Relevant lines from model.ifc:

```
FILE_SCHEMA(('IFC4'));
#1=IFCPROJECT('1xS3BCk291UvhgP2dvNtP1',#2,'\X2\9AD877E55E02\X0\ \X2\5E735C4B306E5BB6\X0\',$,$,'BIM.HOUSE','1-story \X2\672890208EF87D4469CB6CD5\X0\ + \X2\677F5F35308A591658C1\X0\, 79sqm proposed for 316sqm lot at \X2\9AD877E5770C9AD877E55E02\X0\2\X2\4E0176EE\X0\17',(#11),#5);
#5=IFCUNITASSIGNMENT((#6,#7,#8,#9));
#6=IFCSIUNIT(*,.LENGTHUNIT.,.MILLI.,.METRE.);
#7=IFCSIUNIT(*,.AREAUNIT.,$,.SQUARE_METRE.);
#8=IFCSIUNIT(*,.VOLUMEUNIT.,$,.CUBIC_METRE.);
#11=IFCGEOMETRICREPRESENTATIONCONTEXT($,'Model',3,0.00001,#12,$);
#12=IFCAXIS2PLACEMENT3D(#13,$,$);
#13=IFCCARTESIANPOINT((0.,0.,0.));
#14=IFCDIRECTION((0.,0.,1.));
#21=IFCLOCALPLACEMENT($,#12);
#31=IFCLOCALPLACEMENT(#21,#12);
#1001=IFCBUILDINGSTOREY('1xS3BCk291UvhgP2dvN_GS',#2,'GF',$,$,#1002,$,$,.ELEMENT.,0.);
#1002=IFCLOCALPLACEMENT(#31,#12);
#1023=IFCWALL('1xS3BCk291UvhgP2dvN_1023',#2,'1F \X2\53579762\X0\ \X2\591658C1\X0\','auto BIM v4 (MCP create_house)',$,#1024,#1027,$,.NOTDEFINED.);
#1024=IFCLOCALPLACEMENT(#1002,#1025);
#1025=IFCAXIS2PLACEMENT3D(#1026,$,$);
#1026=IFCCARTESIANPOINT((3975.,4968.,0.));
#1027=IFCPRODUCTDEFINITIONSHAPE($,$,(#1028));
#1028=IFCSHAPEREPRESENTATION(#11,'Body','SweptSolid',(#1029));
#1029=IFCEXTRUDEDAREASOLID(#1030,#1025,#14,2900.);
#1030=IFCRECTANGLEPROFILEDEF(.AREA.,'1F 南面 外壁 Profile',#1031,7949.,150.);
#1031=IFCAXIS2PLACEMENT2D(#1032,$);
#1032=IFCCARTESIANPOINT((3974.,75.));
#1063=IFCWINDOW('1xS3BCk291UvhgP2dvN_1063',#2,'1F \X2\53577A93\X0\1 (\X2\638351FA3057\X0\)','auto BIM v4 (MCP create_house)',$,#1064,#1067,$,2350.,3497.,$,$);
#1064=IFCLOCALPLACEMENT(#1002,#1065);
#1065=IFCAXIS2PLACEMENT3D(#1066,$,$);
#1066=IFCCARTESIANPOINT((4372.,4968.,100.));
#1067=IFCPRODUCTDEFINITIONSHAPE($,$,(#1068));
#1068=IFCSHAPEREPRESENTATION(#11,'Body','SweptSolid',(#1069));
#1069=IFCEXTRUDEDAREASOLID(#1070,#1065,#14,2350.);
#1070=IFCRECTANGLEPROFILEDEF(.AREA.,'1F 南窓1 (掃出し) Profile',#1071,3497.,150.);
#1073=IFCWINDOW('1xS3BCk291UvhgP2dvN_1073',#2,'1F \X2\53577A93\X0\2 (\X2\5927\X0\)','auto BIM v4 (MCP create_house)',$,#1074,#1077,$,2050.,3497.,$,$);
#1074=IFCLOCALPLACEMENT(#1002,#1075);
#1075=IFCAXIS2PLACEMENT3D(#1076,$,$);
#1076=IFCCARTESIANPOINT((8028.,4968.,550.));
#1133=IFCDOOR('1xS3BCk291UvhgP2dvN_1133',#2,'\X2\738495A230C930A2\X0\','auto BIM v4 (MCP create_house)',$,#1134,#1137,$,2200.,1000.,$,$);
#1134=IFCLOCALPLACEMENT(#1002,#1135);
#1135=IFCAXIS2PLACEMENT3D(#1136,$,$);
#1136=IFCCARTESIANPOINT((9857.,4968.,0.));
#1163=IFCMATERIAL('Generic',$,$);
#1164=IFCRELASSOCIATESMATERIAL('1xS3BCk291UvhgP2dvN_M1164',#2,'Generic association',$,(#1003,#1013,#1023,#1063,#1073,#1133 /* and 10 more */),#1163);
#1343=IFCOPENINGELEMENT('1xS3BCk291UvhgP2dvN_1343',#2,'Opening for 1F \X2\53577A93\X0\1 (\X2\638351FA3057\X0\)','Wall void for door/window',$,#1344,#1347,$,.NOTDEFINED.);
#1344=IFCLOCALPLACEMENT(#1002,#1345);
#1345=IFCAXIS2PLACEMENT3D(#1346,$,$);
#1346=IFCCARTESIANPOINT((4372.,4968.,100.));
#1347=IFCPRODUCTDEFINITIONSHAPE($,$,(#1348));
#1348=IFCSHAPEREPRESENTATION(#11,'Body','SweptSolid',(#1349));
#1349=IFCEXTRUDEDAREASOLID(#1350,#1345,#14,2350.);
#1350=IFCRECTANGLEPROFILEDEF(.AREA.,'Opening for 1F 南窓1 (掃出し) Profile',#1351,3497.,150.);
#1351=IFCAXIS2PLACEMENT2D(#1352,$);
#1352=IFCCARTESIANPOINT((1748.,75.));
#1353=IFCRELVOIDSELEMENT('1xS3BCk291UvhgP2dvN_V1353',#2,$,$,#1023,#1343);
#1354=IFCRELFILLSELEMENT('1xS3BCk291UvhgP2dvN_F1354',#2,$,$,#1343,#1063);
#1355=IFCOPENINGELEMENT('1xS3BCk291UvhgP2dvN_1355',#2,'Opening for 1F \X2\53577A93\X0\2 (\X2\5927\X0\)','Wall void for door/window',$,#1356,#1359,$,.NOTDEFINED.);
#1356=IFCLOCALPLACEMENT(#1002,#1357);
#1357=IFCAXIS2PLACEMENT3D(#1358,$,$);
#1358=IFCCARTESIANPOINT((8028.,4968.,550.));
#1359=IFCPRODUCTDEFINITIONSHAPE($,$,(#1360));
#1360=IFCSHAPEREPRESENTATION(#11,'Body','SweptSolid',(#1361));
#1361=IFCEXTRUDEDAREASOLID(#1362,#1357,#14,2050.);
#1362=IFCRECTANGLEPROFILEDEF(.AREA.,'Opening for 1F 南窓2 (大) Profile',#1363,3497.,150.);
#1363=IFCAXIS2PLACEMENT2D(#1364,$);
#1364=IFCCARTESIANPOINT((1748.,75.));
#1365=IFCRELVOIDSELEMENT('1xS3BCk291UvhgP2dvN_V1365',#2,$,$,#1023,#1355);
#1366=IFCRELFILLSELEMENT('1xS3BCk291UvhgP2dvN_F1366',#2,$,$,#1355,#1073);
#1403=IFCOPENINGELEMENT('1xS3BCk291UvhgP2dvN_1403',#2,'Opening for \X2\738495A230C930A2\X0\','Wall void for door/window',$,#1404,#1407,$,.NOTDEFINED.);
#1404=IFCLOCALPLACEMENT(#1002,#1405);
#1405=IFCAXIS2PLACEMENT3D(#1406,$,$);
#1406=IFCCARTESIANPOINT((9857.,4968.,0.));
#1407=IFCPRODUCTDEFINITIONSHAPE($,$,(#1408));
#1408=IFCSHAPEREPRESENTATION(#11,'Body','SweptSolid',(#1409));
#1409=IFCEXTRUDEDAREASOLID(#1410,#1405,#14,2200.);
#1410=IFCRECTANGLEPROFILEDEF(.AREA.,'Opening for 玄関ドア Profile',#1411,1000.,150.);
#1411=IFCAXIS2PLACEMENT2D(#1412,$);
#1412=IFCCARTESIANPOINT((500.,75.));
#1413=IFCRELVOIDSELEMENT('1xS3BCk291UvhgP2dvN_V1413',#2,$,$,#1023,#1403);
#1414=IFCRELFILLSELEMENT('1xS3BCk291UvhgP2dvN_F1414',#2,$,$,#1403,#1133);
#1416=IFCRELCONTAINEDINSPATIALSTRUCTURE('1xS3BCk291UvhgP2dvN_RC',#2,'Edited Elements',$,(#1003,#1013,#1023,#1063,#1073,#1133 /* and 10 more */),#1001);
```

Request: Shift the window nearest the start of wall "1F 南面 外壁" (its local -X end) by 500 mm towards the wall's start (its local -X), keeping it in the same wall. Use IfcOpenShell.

```python
import ifcopenshell
import ifcopenshell.api.geometry
import ifcopenshell.util.placement

model = ifcopenshell.open("model.ifc")

window = model.by_id(1063)
opening = window.FillsVoids[0].RelatingOpeningElement
wall = opening.VoidsElements[0].RelatingBuildingElement

wall_matrix = ifcopenshell.util.placement.get_local_placement(wall.ObjectPlacement)
shift = wall_matrix[:3, 0] * -500.0
before = ifcopenshell.util.placement.get_local_placement(window.ObjectPlacement)[:3, 3].copy()

# The window is not placed relative to its opening, so move both.
for product in (opening, window):
    matrix = ifcopenshell.util.placement.get_local_placement(product.ObjectPlacement)
    matrix[:3, 3] += shift
    ifcopenshell.api.geometry.edit_object_placement(model, product=product, matrix=matrix, is_si=False)

after = ifcopenshell.util.placement.get_local_placement(window.ObjectPlacement)[:3, 3]
print("window moved by", (after - before).round(3) + 0.0)

model.write("model_edited.ifc")
```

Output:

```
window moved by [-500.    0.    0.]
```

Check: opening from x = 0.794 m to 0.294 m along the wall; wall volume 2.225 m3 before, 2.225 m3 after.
